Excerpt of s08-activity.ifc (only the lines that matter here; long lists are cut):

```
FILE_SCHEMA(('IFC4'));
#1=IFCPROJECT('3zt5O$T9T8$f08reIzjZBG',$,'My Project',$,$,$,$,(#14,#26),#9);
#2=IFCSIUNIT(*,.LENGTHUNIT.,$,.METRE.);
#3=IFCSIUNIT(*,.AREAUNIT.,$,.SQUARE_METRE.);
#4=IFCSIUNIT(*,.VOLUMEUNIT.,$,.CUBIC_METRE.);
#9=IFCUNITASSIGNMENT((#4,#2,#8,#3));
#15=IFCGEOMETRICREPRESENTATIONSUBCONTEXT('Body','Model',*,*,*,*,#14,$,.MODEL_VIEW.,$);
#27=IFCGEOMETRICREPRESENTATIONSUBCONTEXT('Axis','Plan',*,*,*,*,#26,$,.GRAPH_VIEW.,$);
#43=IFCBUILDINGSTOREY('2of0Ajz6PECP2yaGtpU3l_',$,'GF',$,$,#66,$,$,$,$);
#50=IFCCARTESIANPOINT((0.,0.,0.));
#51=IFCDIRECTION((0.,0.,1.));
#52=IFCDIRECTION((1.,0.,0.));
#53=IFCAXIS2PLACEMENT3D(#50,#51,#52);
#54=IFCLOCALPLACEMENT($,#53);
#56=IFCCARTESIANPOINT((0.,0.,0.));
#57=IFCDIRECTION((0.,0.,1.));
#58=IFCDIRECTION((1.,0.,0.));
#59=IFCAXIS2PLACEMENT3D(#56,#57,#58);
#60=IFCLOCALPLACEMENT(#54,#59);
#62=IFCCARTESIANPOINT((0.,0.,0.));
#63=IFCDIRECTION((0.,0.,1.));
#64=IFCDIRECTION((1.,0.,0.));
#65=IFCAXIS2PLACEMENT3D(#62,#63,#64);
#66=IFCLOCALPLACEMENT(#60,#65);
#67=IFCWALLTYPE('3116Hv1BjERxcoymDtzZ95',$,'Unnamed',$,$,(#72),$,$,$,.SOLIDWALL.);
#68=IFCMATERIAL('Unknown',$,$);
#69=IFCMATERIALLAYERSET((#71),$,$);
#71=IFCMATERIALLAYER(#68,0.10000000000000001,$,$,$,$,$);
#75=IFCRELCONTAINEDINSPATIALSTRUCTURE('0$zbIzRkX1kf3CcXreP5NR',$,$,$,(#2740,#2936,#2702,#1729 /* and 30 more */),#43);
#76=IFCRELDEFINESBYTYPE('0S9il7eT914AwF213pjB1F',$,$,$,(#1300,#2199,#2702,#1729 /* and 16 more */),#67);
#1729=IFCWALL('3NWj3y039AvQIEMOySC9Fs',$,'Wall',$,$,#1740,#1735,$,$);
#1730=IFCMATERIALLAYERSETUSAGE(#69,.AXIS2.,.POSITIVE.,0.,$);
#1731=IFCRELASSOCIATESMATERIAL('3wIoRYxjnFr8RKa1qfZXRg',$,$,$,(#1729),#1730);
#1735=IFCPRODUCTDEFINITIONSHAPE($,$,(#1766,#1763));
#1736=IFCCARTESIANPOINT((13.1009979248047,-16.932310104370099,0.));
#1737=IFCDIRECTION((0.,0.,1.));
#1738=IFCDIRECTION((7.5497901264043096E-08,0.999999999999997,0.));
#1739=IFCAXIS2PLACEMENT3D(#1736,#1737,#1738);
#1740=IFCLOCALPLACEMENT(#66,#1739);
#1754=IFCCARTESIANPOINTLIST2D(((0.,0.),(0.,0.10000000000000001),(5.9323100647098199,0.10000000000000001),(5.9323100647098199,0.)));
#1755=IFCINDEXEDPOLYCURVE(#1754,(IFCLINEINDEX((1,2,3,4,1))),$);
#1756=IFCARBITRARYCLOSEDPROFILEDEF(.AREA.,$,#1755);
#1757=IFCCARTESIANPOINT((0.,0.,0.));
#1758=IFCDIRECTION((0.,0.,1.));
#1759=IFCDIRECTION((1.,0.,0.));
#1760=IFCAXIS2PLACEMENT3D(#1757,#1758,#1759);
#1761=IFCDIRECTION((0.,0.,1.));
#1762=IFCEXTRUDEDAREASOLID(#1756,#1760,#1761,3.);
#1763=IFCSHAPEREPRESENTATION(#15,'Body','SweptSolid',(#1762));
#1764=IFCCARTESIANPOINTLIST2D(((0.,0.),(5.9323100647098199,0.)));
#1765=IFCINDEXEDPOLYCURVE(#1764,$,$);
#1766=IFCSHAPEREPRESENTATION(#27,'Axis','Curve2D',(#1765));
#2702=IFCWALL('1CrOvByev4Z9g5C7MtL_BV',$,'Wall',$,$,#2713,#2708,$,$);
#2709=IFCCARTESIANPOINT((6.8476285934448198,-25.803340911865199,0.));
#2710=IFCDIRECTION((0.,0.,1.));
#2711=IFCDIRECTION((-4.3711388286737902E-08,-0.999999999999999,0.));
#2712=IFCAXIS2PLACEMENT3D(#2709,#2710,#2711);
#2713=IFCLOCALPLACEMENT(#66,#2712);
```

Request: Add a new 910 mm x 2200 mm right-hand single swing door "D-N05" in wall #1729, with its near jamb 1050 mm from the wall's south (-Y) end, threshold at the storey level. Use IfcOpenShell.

```python
import numpy as np
import ifcopenshell
import ifcopenshell.api.feature
import ifcopenshell.api.geometry
import ifcopenshell.api.root
import ifcopenshell.api.spatial
import ifcopenshell.geom
import ifcopenshell.util.element
import ifcopenshell.util.placement
import ifcopenshell.util.representation
import ifcopenshell.util.shape
import ifcopenshell.util.unit

model = ifcopenshell.open("s08-activity.ifc")
unit_scale = ifcopenshell.util.unit.calculate_unit_scale(model)
settings = ifcopenshell.geom.settings()


def volume(element):
    """Net volume in cubic metres, openings subtracted."""
    shape = ifcopenshell.geom.create_shape(settings, element)
    return ifcopenshell.util.shape.get_volume(shape.geometry)


wall = model.by_guid("3NWj3y039AvQIEMOySC9Fs")
storey = ifcopenshell.util.element.get_container(wall, ifc_class="IfcBuildingStorey")
context = ifcopenshell.util.representation.get_context(model, "Model", "Body", "MODEL_VIEW")
before = volume(wall)

width, height, from_end, sill = 0.91, 2.2, 1.05, 0.0  # metres

# The wall runs along its own X axis, and the end named is its -X end.
wall_shape = ifcopenshell.geom.create_shape(settings, wall)
x, y, z = ifcopenshell.util.shape.get_vertices(wall_shape.geometry).T
start = x.min() + from_end
face, thickness = float(y.min()), float(y.max() - y.min())
wall_matrix = ifcopenshell.util.placement.get_local_placement(wall.ObjectPlacement)
level = ifcopenshell.util.placement.get_local_placement(storey.ObjectPlacement)[2, 3]


def in_wall(x, y):
    """Placement at x, y metres in the wall's axes, at sill height."""
    matrix = wall_matrix.copy()
    matrix[:, 3] = wall_matrix @ np.array([x / unit_scale, y / unit_scale, 0.0, 1.0])
    matrix[2, 3] = level + sill / unit_scale
    return matrix


# Opening: a box that overshoots both wall faces by 50 mm.
opening = ifcopenshell.api.root.create_entity(model, ifc_class="IfcOpeningElement", predefined_type="OPENING")
box = ifcopenshell.api.geometry.add_wall_representation(
    model, context=context, length=width, height=height, thickness=thickness + 0.1
)
ifcopenshell.api.geometry.assign_representation(model, product=opening, representation=box)
ifcopenshell.api.geometry.edit_object_placement(model, product=opening, matrix=in_wall(start, face - 0.05), is_si=False)
ifcopenshell.api.feature.add_feature(model, feature=opening, element=wall)

door = ifcopenshell.api.root.create_entity(model, ifc_class="IfcDoor", name="D-N05", predefined_type="DOOR")
door.OverallWidth, door.OverallHeight = width / unit_scale, height / unit_scale
door.OperationType = "SINGLE_SWING_RIGHT"
body = ifcopenshell.api.geometry.add_door_representation(
    model,
    context=context,
    overall_width=door.OverallWidth,
    overall_height=door.OverallHeight,
    operation_type="SINGLE_SWING_RIGHT",
    lining_properties={"LiningDepth": thickness / unit_scale, "ThresholdDepth": thickness / unit_scale},
)
ifcopenshell.api.geometry.assign_representation(model, product=door, representation=body)
ifcopenshell.api.spatial.assign_container(model, products=[door], relating_structure=storey)
ifcopenshell.api.feature.add_filling(model, opening=opening, element=door)

# The lining spans the wall, so the door starts at the wall face.
ifcopenshell.api.geometry.edit_object_placement(model, product=door, matrix=in_wall(start, face), is_si=False)

after = volume(wall)

print(f"wall volume {before:.3f} -> {after:.3f} m3")

model.write("s08-activity_rev.ifc")
```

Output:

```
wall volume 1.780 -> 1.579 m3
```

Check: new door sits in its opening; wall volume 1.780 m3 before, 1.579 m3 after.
